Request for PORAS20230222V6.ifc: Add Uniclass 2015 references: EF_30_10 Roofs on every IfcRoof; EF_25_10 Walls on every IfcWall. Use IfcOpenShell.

First a look at what the model holds.

```python
import ifcopenshell

model = ifcopenshell.open("PORAS20230222V6.ifc")
print(model.schema)
print("classifications:", [c.Name for c in model.by_type("IfcClassification")])
for ifc_class in ("IfcDoor", "IfcRoof", "IfcStair", "IfcWall", "IfcWindow"):
    print(ifc_class, len(model.by_type(ifc_class)))
```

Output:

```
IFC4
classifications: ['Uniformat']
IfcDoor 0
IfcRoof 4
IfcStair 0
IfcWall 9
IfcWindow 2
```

```python
import ifcopenshell
import ifcopenshell.api.classification

model = ifcopenshell.open("PORAS20230222V6.ifc")

system = ifcopenshell.api.classification.add_classification(model, classification="Uniclass 2015")

codes = {
    "IfcRoof": ("EF_30_10", "Roofs"),
    "IfcWall": ("EF_25_10", "Walls"),
}
for ifc_class, (code, name) in codes.items():
    products = model.by_type(ifc_class)
    ifcopenshell.api.classification.add_reference(
        model, products=products, classification=system, identification=code, name=name
    )
    print(code, len(products))

model.write("PORAS20230222V6_rev.ifc")
```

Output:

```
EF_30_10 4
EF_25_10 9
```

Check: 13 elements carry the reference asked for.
